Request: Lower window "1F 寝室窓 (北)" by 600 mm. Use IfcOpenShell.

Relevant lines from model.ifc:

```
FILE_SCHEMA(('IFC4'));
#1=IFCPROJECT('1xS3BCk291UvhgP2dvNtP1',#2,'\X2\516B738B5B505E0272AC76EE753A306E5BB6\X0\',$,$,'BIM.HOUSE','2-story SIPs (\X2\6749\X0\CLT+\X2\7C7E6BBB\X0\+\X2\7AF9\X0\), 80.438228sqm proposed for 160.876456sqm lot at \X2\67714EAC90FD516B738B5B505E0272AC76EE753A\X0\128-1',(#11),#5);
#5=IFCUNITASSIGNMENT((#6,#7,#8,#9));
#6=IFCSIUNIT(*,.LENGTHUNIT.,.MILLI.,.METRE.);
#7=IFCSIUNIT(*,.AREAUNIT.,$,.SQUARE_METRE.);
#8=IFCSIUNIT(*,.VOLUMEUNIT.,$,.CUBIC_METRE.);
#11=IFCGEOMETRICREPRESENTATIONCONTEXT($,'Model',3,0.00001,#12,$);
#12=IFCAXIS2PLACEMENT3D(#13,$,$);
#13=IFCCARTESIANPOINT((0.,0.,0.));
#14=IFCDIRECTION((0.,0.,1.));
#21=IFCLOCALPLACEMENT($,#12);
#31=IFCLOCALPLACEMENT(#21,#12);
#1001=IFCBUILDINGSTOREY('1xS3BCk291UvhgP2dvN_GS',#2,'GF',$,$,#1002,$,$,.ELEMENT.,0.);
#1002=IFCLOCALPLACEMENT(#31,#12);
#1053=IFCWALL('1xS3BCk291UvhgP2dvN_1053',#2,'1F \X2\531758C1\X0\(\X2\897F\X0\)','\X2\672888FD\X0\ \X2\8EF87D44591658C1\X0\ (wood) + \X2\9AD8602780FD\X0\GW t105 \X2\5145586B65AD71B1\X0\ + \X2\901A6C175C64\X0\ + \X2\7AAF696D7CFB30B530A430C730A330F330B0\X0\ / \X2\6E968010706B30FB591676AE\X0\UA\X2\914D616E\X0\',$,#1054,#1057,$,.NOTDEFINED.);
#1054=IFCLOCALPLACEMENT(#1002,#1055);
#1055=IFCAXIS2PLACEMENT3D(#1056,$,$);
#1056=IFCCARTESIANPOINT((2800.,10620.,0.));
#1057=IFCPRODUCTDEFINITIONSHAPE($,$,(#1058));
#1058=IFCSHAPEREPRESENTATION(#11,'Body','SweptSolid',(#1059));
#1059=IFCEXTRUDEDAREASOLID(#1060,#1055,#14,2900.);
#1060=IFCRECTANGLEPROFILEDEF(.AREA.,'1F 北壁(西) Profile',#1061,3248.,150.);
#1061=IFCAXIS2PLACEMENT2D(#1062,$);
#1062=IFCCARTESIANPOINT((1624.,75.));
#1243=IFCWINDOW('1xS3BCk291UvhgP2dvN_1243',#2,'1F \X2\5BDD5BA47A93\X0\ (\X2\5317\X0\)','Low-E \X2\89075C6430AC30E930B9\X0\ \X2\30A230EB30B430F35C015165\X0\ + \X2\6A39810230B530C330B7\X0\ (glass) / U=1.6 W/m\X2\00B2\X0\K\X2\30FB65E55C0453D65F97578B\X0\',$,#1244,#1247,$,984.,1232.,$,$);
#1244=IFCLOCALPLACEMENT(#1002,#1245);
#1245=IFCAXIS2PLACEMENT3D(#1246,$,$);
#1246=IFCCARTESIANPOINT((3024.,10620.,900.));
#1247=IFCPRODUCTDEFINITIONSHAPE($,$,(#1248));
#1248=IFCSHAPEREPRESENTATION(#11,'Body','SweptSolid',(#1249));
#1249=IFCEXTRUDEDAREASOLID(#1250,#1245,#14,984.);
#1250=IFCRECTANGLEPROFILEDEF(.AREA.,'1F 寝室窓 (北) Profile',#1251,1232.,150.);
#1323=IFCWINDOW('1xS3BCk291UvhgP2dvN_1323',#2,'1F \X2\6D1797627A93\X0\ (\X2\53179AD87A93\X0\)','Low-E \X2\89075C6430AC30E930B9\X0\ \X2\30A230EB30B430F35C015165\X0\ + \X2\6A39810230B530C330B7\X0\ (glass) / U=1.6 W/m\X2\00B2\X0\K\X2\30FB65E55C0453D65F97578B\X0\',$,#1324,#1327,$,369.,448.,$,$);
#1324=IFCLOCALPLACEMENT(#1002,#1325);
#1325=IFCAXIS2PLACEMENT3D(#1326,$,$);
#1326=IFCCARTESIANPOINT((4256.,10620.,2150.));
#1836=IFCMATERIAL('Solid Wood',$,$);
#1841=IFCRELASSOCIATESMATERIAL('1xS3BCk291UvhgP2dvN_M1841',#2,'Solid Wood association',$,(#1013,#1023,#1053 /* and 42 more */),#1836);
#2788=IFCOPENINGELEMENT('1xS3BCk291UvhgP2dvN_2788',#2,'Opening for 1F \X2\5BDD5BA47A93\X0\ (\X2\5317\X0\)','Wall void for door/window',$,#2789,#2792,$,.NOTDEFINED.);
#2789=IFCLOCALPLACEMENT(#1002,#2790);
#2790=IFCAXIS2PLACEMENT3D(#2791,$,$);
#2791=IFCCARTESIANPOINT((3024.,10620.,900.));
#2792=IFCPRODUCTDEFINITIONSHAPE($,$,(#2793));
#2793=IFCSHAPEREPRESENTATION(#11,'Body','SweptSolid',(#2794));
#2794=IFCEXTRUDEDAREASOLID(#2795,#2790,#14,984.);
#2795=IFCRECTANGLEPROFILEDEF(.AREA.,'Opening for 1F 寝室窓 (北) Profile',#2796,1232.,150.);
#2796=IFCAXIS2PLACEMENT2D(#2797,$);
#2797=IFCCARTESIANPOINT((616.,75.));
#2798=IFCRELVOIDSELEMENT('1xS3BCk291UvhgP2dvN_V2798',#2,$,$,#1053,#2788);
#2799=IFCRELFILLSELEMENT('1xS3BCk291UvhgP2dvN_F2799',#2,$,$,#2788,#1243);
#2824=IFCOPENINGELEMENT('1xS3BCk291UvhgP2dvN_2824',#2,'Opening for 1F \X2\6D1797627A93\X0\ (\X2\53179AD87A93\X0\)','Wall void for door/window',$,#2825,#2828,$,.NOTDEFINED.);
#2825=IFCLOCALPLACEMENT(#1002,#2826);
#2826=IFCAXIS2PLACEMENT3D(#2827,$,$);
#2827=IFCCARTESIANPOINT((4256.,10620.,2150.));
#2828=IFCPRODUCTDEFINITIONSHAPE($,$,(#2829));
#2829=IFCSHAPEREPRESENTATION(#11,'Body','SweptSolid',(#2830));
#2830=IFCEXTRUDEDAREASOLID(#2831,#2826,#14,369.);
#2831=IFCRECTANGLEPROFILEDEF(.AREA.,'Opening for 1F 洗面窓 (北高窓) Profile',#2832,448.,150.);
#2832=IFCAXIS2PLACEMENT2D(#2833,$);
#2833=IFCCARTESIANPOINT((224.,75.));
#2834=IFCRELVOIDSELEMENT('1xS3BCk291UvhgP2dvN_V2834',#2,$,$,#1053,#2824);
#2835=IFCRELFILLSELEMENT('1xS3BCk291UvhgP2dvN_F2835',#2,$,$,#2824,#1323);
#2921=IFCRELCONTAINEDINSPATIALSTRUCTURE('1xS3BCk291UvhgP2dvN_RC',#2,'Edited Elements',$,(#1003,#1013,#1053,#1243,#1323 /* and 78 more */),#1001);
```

```python
import numpy as np
import ifcopenshell
import ifcopenshell.api.geometry
import ifcopenshell.util.placement
import ifcopenshell.util.unit

model = ifcopenshell.open("model.ifc")
unit_scale = ifcopenshell.util.unit.calculate_unit_scale(model)

window = model.by_id(1243)
opening = window.FillsVoids[0].RelatingOpeningElement
dz = -0.6 / unit_scale

shift = np.array([0.0, 0.0, dz])
# The window is not placed relative to its opening, so move both.
for product in (opening, window):
    matrix = ifcopenshell.util.placement.get_local_placement(product.ObjectPlacement)
    matrix[:3, 3] += shift
    ifcopenshell.api.geometry.edit_object_placement(model, product=product, matrix=matrix, is_si=False)

print(f"moved by {dz * unit_scale:+.3f} m")

model.write("model_rev.ifc")
```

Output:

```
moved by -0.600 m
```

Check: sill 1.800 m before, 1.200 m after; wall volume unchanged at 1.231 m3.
